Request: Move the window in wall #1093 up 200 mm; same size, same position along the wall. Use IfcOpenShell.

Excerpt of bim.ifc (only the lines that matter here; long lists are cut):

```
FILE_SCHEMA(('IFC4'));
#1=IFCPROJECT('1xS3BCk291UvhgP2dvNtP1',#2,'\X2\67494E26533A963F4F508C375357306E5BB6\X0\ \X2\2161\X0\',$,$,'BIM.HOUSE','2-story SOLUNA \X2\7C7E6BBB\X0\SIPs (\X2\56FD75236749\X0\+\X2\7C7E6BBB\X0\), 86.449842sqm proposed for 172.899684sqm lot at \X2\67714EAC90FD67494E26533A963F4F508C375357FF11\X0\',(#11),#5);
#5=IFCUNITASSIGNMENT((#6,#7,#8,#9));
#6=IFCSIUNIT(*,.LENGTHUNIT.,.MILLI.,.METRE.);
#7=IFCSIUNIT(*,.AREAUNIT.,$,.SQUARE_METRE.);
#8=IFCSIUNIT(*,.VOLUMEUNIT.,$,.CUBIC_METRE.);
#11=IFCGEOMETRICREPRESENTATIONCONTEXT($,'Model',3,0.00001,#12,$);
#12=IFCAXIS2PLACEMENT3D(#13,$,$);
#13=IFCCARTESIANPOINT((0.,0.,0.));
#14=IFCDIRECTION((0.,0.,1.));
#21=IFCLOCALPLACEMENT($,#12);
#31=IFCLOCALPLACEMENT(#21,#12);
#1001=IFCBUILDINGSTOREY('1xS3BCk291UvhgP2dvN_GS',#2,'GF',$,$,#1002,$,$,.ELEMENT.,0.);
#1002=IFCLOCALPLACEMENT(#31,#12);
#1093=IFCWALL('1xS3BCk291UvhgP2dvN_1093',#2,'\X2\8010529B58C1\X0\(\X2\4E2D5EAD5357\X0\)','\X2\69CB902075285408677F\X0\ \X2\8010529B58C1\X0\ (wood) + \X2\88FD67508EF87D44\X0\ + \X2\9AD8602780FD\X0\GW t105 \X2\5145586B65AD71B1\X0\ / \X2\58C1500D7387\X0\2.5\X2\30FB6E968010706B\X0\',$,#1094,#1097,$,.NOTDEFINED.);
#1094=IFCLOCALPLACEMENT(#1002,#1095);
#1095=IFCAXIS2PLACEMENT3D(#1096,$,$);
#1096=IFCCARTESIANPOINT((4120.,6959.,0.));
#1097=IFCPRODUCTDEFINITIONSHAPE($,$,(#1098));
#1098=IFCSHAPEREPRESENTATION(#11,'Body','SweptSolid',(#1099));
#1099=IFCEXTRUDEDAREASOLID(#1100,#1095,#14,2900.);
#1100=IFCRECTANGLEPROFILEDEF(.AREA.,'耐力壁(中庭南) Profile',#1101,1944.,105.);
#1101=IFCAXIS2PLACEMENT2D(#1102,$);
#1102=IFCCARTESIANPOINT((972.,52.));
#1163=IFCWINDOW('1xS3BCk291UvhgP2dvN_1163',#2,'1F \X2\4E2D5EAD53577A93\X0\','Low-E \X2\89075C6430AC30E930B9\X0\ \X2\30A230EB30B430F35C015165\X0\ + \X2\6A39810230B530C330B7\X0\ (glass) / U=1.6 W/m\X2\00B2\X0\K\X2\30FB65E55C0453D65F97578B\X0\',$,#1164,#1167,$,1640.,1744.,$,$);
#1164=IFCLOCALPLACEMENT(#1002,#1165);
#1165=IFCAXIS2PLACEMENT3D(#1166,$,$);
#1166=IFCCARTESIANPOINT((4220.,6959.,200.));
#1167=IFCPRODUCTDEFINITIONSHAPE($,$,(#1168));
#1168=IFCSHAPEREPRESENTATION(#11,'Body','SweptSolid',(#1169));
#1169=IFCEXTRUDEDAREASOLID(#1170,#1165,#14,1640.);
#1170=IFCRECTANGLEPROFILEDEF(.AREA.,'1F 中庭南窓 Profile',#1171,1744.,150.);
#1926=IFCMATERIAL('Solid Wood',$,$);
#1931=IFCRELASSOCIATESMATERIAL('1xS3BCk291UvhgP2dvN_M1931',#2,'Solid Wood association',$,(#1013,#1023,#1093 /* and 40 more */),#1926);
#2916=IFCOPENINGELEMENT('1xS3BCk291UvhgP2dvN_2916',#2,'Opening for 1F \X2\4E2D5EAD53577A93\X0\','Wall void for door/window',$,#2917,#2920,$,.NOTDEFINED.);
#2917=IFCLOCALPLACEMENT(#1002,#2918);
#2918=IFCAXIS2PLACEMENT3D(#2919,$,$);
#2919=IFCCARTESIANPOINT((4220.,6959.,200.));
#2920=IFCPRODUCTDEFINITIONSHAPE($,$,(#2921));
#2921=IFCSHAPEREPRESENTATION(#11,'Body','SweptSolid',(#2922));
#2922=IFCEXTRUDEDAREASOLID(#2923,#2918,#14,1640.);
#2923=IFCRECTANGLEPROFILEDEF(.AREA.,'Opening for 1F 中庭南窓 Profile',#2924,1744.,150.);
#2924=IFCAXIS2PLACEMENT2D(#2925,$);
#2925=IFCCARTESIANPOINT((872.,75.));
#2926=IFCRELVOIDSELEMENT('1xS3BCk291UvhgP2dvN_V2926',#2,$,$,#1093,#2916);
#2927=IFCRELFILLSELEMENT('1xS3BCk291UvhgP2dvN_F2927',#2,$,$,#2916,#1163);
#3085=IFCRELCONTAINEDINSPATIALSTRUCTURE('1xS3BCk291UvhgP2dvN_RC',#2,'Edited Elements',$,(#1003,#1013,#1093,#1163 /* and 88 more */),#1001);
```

```python
import numpy as np
import ifcopenshell
import ifcopenshell.api.geometry
import ifcopenshell.util.placement
import ifcopenshell.util.unit

model = ifcopenshell.open("bim.ifc")
unit_scale = ifcopenshell.util.unit.calculate_unit_scale(model)

window = model.by_guid("1xS3BCk291UvhgP2dvN_1163")
opening = window.FillsVoids[0].RelatingOpeningElement
dz = 200.0

shift = np.array([0.0, 0.0, dz])
# The window is not placed relative to its opening, so move both.
for product in (opening, window):
    matrix = ifcopenshell.util.placement.get_local_placement(product.ObjectPlacement)
    matrix[:3, 3] += shift
    ifcopenshell.api.geometry.edit_object_placement(model, product=product, matrix=matrix, is_si=False)

print(f"moved by {dz * unit_scale:+.3f} m")

model.write("bim_rev.ifc")
```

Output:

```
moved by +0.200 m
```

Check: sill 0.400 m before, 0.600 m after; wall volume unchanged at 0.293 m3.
